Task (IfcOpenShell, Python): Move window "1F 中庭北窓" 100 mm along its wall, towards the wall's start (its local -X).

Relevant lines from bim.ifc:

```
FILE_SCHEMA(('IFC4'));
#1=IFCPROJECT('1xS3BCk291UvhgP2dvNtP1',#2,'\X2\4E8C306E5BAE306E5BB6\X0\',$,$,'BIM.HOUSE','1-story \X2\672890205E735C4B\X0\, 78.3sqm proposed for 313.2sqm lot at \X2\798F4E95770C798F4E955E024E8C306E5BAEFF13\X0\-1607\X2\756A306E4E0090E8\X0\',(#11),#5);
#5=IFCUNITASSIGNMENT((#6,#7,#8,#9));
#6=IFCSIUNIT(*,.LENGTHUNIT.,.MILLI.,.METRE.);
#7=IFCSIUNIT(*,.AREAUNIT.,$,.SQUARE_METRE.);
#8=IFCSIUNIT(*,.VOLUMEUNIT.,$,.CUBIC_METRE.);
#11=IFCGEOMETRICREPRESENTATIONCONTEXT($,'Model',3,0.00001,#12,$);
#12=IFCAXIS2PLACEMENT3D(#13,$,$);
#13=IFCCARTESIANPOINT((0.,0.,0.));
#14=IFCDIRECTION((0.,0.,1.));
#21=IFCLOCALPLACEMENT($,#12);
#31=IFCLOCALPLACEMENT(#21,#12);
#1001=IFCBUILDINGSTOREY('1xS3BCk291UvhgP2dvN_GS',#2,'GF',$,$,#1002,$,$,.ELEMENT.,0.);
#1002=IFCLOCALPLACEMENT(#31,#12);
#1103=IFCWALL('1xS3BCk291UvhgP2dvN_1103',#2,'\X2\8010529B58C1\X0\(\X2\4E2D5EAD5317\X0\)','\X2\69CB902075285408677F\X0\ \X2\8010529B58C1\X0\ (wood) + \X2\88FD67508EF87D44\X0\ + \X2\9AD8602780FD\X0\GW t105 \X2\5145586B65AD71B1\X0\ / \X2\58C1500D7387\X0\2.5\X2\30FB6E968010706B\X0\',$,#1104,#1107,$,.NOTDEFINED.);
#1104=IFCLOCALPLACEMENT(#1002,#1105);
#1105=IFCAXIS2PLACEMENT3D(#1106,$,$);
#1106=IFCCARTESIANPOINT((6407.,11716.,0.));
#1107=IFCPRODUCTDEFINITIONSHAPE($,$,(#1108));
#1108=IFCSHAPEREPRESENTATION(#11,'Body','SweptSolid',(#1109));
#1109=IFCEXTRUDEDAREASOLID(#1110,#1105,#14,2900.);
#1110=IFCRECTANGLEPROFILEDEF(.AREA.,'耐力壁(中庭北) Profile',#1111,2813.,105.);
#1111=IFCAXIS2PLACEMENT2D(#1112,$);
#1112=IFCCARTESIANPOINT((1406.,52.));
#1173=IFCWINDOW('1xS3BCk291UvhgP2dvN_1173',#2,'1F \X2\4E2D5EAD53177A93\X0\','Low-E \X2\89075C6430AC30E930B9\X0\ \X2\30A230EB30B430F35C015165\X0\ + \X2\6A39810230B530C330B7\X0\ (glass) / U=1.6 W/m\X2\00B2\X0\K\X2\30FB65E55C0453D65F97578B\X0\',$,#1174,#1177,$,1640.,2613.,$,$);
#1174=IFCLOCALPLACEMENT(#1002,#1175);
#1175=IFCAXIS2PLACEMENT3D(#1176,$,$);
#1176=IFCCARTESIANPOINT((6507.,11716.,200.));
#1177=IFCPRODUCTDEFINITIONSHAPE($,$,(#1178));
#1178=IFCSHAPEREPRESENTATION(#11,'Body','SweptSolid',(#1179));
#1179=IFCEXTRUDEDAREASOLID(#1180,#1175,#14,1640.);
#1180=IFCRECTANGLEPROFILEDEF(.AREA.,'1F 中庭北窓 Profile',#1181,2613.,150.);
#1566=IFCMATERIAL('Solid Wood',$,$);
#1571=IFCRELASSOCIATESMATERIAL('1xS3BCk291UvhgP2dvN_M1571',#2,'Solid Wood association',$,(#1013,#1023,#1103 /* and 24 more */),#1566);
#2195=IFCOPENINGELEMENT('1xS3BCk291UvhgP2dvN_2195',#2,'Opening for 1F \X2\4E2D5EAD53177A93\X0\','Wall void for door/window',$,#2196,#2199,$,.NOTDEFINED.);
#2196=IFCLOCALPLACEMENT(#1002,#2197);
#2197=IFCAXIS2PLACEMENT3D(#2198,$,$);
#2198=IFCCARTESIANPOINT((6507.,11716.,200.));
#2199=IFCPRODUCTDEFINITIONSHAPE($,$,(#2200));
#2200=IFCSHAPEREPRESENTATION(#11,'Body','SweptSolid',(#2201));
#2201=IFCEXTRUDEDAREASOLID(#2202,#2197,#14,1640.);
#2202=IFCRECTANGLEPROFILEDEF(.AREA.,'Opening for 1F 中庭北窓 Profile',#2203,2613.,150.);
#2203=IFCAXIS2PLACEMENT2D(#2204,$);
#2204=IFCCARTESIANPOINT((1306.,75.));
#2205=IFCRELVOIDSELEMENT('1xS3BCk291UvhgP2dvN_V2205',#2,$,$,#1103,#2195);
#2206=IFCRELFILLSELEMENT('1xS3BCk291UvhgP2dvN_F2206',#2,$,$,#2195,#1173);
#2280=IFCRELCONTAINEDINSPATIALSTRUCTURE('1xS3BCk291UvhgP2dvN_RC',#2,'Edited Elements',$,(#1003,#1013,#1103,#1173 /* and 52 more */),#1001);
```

```python
import ifcopenshell
import ifcopenshell.api.geometry
import ifcopenshell.util.placement
import ifcopenshell.util.unit

model = ifcopenshell.open("bim.ifc")
unit_scale = ifcopenshell.util.unit.calculate_unit_scale(model)

window = model.by_guid("1xS3BCk291UvhgP2dvN_1173")
opening = window.FillsVoids[0].RelatingOpeningElement
wall = opening.VoidsElements[0].RelatingBuildingElement

wall_matrix = ifcopenshell.util.placement.get_local_placement(wall.ObjectPlacement)
shift = wall_matrix[:3, 0] * -0.1 / unit_scale
before = ifcopenshell.util.placement.get_local_placement(window.ObjectPlacement)[:3, 3].copy()

# The window is not placed relative to its opening, so move both.
for product in (opening, window):
    matrix = ifcopenshell.util.placement.get_local_placement(product.ObjectPlacement)
    matrix[:3, 3] += shift
    ifcopenshell.api.geometry.edit_object_placement(model, product=product, matrix=matrix, is_si=False)

after = ifcopenshell.util.placement.get_local_placement(window.ObjectPlacement)[:3, 3]
print("window moved by", (after - before).round(3) + 0.0)

model.write("bim_edited.ifc")
```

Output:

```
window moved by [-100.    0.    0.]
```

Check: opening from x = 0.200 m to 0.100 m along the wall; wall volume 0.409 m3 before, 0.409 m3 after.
